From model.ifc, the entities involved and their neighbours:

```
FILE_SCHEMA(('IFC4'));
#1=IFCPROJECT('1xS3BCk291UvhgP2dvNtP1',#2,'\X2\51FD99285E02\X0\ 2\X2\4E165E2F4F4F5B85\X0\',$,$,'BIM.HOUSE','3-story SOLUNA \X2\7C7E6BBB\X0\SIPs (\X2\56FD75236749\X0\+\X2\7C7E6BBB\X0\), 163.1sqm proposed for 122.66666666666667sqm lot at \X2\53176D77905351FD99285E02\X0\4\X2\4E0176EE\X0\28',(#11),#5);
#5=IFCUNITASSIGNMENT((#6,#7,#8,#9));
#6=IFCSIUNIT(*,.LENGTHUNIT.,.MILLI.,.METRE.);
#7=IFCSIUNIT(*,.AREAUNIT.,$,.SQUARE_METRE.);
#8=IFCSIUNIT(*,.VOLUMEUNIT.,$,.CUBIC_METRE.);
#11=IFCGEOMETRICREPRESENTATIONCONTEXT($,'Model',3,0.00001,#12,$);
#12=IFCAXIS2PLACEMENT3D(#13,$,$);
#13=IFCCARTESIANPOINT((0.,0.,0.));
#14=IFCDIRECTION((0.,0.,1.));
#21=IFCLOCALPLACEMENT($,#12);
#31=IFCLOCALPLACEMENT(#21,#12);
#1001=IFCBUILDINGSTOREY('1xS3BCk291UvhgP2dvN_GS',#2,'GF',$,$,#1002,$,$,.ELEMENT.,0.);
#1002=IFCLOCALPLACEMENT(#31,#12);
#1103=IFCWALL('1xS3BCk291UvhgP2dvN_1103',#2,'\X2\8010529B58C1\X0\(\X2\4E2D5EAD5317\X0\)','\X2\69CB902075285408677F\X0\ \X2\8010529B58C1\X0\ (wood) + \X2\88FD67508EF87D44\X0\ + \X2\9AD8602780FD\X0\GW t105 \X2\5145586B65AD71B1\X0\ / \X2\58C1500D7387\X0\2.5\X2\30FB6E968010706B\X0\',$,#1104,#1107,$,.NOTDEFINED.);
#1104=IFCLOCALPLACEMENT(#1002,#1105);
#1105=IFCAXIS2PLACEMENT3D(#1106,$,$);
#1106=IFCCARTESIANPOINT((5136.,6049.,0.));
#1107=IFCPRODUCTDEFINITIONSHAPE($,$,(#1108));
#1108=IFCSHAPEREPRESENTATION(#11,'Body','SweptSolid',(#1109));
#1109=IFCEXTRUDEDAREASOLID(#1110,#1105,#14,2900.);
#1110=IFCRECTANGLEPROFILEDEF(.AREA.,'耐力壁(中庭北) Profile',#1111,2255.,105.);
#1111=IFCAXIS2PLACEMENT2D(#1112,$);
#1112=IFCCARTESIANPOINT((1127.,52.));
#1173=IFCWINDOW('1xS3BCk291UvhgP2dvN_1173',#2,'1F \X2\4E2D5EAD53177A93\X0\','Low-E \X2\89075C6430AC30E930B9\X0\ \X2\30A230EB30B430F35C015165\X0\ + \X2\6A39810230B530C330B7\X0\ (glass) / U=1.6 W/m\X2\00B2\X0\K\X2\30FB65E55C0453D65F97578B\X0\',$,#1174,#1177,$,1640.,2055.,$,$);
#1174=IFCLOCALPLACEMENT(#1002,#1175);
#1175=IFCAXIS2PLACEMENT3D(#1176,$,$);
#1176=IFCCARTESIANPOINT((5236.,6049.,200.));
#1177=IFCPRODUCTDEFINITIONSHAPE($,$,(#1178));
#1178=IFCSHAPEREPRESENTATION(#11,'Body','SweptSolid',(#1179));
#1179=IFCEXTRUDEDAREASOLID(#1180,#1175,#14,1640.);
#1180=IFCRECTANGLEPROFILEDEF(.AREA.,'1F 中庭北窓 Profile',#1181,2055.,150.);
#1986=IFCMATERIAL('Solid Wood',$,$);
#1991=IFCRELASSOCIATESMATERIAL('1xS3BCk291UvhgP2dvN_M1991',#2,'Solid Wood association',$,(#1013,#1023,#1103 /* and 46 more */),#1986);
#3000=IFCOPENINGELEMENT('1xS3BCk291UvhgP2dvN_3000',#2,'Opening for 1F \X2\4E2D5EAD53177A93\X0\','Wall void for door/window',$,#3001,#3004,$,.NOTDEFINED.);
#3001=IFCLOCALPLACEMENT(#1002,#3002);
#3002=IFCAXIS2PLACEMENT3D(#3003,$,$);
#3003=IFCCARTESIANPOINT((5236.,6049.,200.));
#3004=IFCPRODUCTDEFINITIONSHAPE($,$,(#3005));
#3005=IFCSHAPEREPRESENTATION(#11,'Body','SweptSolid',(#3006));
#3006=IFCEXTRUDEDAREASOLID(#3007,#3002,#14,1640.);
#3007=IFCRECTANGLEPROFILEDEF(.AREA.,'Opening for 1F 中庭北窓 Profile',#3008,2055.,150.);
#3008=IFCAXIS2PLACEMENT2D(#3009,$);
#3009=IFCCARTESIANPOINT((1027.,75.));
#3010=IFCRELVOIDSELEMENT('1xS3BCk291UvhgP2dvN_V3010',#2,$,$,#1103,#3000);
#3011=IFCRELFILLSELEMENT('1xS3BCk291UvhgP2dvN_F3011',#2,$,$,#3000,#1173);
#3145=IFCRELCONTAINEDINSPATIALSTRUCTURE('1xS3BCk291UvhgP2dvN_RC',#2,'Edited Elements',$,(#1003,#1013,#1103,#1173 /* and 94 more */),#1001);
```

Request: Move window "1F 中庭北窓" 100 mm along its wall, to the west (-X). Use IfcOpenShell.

```python
import ifcopenshell
import ifcopenshell.api.geometry
import ifcopenshell.util.placement

model = ifcopenshell.open("model.ifc")

window = model.by_guid("1xS3BCk291UvhgP2dvN_1173")
opening = window.FillsVoids[0].RelatingOpeningElement
wall = opening.VoidsElements[0].RelatingBuildingElement

wall_matrix = ifcopenshell.util.placement.get_local_placement(wall.ObjectPlacement)
shift = wall_matrix[:3, 0] * -100.0
before = ifcopenshell.util.placement.get_local_placement(window.ObjectPlacement)[:3, 3].copy()

# The window is not placed relative to its opening, so move both.
for product in (opening, window):
    matrix = ifcopenshell.util.placement.get_local_placement(product.ObjectPlacement)
    matrix[:3, 3] += shift
    ifcopenshell.api.geometry.edit_object_placement(model, product=product, matrix=matrix, is_si=False)

after = ifcopenshell.util.placement.get_local_placement(window.ObjectPlacement)[:3, 3]
print("window moved by", (after - before).round(3) + 0.0)

model.write("model_v2.ifc")
```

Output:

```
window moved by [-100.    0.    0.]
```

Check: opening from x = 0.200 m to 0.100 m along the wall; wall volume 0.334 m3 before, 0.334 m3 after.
